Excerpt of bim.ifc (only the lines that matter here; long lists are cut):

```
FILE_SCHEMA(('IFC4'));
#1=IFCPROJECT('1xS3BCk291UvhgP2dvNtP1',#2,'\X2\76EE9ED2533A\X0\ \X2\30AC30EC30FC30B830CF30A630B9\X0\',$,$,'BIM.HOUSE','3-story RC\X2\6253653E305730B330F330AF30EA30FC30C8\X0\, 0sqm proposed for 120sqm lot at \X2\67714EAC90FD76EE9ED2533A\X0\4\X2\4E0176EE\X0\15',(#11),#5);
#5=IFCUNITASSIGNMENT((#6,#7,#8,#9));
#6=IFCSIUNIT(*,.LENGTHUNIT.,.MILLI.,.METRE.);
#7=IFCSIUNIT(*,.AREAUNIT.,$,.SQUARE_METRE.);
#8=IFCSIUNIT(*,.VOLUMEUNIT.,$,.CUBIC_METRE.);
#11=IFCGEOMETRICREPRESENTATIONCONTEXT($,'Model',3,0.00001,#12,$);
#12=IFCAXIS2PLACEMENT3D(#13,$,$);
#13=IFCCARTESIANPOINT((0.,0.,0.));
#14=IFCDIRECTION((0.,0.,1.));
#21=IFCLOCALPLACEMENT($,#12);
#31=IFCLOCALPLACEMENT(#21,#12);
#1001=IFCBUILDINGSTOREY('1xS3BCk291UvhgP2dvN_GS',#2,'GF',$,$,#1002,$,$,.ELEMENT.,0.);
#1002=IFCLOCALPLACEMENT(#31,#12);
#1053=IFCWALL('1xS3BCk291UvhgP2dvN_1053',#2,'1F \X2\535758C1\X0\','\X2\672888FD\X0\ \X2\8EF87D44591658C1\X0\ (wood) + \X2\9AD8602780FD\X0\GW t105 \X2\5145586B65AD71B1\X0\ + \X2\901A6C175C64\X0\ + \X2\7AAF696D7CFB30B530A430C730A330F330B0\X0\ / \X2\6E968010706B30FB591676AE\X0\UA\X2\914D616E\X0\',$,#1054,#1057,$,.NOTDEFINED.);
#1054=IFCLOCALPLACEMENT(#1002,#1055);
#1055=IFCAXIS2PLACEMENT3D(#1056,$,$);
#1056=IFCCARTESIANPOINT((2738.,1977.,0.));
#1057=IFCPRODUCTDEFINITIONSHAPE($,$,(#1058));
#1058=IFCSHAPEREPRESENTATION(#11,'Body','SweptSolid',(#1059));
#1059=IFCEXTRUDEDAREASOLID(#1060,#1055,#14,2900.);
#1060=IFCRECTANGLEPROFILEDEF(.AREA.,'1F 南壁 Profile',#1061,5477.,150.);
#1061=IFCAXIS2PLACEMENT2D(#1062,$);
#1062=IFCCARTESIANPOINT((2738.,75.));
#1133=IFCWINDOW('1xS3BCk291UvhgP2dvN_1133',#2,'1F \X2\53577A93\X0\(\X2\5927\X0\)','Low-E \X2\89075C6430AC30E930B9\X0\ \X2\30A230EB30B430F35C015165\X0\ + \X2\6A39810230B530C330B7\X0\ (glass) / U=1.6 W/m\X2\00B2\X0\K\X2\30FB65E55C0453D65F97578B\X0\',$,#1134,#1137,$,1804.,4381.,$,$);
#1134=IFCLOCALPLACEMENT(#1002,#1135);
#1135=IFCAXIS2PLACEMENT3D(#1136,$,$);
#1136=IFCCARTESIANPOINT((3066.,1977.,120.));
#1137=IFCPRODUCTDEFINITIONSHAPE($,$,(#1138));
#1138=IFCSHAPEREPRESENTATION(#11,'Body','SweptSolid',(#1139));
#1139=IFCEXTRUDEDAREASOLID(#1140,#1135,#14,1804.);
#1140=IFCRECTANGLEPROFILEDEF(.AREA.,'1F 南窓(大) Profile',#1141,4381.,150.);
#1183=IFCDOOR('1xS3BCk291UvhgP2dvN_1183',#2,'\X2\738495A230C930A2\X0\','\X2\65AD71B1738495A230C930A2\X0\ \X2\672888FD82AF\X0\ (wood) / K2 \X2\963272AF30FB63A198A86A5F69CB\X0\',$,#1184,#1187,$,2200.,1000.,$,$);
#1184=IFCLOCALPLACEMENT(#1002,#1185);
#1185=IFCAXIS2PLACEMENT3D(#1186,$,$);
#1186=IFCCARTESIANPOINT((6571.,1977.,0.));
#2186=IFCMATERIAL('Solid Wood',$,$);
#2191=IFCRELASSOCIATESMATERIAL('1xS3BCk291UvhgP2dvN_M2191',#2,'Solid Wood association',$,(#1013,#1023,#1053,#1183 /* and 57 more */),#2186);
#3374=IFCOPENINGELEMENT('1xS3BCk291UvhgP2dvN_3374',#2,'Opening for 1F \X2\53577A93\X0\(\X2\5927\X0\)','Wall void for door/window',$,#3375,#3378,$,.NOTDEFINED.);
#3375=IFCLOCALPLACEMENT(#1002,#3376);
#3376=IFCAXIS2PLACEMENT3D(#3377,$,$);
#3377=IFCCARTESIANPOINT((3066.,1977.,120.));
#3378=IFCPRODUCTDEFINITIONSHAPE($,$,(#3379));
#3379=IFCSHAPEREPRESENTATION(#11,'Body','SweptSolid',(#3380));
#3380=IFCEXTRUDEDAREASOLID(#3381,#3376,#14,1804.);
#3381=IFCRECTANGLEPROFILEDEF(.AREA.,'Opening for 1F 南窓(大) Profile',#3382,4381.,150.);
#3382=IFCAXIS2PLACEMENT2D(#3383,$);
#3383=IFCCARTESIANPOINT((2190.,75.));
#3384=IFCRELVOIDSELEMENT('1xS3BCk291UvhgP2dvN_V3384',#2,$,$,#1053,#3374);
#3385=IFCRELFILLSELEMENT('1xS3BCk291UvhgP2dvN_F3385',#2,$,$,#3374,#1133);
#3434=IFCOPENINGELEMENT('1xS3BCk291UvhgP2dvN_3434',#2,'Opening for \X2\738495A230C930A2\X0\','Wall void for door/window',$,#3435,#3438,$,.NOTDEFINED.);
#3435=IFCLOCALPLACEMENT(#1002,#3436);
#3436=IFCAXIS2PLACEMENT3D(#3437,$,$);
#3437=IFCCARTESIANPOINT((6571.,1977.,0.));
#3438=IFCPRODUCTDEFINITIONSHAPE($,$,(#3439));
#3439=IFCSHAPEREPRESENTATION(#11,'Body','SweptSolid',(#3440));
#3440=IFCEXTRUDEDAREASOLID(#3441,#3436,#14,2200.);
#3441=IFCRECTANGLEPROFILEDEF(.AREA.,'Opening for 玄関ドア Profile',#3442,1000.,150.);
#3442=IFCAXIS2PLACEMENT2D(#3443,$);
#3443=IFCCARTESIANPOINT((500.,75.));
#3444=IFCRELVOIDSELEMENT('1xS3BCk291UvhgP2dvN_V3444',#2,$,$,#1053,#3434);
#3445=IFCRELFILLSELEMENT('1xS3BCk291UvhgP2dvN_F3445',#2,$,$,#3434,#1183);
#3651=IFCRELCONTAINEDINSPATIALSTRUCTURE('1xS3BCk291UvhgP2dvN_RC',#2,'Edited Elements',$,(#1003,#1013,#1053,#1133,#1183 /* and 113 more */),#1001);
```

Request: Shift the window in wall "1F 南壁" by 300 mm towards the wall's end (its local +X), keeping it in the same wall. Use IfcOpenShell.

```python
import ifcopenshell
import ifcopenshell.api.geometry
import ifcopenshell.util.placement

model = ifcopenshell.open("bim.ifc")

window = model.by_guid("1xS3BCk291UvhgP2dvN_1133")
opening = window.FillsVoids[0].RelatingOpeningElement
wall = opening.VoidsElements[0].RelatingBuildingElement

wall_matrix = ifcopenshell.util.placement.get_local_placement(wall.ObjectPlacement)
shift = wall_matrix[:3, 0] * 300.0
before = ifcopenshell.util.placement.get_local_placement(window.ObjectPlacement)[:3, 3].copy()

# The window is not placed relative to its opening, so move both.
for product in (opening, window):
    matrix = ifcopenshell.util.placement.get_local_placement(product.ObjectPlacement)
    matrix[:3, 3] += shift
    ifcopenshell.api.geometry.edit_object_placement(model, product=product, matrix=matrix, is_si=False)

after = ifcopenshell.util.placement.get_local_placement(window.ObjectPlacement)[:3, 3]
print("window moved by", (after - before).round(3) + 0.0)

model.write("bim-out.ifc")
```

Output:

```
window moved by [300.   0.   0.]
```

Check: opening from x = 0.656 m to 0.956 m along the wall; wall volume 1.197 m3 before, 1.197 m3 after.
